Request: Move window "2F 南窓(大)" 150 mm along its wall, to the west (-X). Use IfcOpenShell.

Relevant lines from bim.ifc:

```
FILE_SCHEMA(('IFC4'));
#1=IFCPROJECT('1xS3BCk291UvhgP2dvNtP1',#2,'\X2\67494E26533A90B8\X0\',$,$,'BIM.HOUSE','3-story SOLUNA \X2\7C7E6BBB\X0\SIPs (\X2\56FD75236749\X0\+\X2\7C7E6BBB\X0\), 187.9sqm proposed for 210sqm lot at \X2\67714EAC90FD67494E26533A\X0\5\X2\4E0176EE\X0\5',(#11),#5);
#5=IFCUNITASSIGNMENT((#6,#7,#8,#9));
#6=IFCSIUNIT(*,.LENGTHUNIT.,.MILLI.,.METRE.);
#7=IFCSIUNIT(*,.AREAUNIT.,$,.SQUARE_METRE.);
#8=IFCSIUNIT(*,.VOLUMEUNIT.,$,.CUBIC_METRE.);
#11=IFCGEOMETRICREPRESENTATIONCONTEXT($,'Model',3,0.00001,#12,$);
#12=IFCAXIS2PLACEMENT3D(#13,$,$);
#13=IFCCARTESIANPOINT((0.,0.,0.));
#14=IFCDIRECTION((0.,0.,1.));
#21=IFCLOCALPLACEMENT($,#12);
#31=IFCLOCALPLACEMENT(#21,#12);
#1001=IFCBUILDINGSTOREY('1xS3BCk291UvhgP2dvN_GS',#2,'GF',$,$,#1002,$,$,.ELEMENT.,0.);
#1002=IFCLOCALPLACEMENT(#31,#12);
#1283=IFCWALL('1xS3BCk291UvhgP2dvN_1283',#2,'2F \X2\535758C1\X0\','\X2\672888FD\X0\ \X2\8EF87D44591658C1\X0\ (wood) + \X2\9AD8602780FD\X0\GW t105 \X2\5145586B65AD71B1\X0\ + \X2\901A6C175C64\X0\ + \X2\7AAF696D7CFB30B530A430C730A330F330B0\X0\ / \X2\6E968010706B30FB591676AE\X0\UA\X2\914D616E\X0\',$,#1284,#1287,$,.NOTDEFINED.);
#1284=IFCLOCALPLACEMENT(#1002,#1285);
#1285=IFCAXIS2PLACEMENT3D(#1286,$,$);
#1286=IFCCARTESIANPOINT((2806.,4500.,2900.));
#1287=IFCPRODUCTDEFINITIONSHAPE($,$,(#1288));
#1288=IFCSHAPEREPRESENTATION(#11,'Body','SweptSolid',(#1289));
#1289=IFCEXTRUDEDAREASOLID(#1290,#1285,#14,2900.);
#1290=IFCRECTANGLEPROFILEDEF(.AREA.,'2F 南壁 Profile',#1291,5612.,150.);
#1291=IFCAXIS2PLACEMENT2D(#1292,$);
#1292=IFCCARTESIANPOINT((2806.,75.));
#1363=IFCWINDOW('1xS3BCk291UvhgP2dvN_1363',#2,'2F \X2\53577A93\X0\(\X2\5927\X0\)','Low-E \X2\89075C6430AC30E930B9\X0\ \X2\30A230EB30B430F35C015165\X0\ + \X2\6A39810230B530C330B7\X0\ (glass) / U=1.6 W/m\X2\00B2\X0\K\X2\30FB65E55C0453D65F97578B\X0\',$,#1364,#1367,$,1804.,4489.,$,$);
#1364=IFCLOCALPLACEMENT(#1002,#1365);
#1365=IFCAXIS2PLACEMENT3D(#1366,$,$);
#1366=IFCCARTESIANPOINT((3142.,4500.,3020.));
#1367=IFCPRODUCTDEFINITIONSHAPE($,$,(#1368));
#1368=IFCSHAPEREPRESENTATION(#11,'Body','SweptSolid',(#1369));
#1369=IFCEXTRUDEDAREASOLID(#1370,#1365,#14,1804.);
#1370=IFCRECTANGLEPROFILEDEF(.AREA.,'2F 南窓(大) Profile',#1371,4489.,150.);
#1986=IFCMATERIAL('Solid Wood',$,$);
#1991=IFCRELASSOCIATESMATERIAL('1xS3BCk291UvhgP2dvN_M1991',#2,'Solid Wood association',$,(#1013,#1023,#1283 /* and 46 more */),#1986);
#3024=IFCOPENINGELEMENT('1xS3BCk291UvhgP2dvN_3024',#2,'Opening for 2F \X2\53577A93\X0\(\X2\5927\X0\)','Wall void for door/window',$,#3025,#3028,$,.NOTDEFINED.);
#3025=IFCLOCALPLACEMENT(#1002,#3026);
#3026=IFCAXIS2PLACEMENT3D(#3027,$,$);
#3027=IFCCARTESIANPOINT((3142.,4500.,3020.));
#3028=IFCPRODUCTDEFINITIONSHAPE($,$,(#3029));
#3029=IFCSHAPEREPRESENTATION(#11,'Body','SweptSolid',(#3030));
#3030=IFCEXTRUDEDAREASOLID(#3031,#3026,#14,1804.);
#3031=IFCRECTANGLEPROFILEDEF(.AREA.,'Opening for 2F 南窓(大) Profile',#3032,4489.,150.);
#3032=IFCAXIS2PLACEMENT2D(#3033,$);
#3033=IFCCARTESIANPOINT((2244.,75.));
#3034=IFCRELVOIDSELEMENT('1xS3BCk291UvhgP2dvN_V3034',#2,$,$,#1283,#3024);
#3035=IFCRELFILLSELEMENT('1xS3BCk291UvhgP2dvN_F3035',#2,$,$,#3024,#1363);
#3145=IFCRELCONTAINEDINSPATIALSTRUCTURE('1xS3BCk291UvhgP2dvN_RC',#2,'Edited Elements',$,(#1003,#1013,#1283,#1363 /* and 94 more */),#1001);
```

```python
import ifcopenshell
import ifcopenshell.api.geometry
import ifcopenshell.util.placement

model = ifcopenshell.open("bim.ifc")

window = model.by_guid("1xS3BCk291UvhgP2dvN_1363")
opening = window.FillsVoids[0].RelatingOpeningElement
wall = opening.VoidsElements[0].RelatingBuildingElement

wall_matrix = ifcopenshell.util.placement.get_local_placement(wall.ObjectPlacement)
shift = wall_matrix[:3, 0] * -150.0
before = ifcopenshell.util.placement.get_local_placement(window.ObjectPlacement)[:3, 3].copy()

# The window is not placed relative to its opening, so move both.
for product in (opening, window):
    matrix = ifcopenshell.util.placement.get_local_placement(product.ObjectPlacement)
    matrix[:3, 3] += shift
    ifcopenshell.api.geometry.edit_object_placement(model, product=product, matrix=matrix, is_si=False)

after = ifcopenshell.util.placement.get_local_placement(window.ObjectPlacement)[:3, 3]
print("window moved by", (after - before).round(3) + 0.0)

model.write("bim_edited.ifc")
```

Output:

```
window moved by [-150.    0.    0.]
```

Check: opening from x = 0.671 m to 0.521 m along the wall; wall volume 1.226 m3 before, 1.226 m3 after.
